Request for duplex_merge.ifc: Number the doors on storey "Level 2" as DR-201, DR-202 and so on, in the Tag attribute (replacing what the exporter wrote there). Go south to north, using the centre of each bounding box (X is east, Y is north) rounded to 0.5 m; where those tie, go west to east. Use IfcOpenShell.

First a look at what the model holds.

```python
import ifcopenshell
import ifcopenshell.util.element
import ifcopenshell.util.placement

model = ifcopenshell.open("duplex_merge.ifc")
print(model.schema)
storey = next(s for s in model.by_type("IfcBuildingStorey") if s.Name == "Level 2")
doors = [e for e in ifcopenshell.util.element.get_decomposition(storey) if e.is_a("IfcDoor")]
for e in sorted(doors, key=lambda e: e.id()):
    origin = ifcopenshell.util.placement.get_local_placement(e.ObjectPlacement)[:3, 3]
    print(e.id(), e.Tag, e.Name, origin.round(2) + 0.0, sep=" | ")
```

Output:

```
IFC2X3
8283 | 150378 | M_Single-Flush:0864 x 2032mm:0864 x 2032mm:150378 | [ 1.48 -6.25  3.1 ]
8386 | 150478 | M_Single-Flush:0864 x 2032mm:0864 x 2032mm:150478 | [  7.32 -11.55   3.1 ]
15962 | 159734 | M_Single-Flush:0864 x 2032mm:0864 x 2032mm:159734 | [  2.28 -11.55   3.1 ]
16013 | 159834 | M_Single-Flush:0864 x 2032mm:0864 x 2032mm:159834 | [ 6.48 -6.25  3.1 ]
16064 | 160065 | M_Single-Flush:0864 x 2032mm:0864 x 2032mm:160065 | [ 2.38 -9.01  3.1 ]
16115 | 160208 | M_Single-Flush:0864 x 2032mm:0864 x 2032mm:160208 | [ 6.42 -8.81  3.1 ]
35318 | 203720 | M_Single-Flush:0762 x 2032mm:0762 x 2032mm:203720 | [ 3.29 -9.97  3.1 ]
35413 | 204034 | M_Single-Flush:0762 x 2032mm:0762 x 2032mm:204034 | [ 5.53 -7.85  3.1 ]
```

```python
import ifcopenshell
import ifcopenshell.geom
import ifcopenshell.util.element
import ifcopenshell.util.shape

model = ifcopenshell.open("duplex_merge.ifc")
settings = ifcopenshell.geom.settings()
settings.set("use-world-coords", True)


def centre(element):
    shape = ifcopenshell.geom.create_shape(settings, element)
    return ifcopenshell.util.shape.get_bbox_centroid(shape.geometry)


storey = next(s for s in model.by_type("IfcBuildingStorey") if s.Name == "Level 2")
doors = [e for e in ifcopenshell.util.element.get_decomposition(storey) if e.is_a("IfcDoor")]

# Insertion points can sit at a corner or the storey origin, so sort by the geometry (in metres).
centres = {e: centre(e) for e in doors}
doors.sort(key=lambda e: (round(centres[e][1] / 0.5), centres[e][0]))

for i, e in enumerate(doors, start=1):
    number = f"DR-2{i:02d}"
    e.Tag = number
    print(e.id(), number)

model.write("duplex_merge_rev.ifc")
```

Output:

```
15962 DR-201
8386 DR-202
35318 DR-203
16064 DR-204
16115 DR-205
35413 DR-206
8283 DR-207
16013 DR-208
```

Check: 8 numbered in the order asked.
